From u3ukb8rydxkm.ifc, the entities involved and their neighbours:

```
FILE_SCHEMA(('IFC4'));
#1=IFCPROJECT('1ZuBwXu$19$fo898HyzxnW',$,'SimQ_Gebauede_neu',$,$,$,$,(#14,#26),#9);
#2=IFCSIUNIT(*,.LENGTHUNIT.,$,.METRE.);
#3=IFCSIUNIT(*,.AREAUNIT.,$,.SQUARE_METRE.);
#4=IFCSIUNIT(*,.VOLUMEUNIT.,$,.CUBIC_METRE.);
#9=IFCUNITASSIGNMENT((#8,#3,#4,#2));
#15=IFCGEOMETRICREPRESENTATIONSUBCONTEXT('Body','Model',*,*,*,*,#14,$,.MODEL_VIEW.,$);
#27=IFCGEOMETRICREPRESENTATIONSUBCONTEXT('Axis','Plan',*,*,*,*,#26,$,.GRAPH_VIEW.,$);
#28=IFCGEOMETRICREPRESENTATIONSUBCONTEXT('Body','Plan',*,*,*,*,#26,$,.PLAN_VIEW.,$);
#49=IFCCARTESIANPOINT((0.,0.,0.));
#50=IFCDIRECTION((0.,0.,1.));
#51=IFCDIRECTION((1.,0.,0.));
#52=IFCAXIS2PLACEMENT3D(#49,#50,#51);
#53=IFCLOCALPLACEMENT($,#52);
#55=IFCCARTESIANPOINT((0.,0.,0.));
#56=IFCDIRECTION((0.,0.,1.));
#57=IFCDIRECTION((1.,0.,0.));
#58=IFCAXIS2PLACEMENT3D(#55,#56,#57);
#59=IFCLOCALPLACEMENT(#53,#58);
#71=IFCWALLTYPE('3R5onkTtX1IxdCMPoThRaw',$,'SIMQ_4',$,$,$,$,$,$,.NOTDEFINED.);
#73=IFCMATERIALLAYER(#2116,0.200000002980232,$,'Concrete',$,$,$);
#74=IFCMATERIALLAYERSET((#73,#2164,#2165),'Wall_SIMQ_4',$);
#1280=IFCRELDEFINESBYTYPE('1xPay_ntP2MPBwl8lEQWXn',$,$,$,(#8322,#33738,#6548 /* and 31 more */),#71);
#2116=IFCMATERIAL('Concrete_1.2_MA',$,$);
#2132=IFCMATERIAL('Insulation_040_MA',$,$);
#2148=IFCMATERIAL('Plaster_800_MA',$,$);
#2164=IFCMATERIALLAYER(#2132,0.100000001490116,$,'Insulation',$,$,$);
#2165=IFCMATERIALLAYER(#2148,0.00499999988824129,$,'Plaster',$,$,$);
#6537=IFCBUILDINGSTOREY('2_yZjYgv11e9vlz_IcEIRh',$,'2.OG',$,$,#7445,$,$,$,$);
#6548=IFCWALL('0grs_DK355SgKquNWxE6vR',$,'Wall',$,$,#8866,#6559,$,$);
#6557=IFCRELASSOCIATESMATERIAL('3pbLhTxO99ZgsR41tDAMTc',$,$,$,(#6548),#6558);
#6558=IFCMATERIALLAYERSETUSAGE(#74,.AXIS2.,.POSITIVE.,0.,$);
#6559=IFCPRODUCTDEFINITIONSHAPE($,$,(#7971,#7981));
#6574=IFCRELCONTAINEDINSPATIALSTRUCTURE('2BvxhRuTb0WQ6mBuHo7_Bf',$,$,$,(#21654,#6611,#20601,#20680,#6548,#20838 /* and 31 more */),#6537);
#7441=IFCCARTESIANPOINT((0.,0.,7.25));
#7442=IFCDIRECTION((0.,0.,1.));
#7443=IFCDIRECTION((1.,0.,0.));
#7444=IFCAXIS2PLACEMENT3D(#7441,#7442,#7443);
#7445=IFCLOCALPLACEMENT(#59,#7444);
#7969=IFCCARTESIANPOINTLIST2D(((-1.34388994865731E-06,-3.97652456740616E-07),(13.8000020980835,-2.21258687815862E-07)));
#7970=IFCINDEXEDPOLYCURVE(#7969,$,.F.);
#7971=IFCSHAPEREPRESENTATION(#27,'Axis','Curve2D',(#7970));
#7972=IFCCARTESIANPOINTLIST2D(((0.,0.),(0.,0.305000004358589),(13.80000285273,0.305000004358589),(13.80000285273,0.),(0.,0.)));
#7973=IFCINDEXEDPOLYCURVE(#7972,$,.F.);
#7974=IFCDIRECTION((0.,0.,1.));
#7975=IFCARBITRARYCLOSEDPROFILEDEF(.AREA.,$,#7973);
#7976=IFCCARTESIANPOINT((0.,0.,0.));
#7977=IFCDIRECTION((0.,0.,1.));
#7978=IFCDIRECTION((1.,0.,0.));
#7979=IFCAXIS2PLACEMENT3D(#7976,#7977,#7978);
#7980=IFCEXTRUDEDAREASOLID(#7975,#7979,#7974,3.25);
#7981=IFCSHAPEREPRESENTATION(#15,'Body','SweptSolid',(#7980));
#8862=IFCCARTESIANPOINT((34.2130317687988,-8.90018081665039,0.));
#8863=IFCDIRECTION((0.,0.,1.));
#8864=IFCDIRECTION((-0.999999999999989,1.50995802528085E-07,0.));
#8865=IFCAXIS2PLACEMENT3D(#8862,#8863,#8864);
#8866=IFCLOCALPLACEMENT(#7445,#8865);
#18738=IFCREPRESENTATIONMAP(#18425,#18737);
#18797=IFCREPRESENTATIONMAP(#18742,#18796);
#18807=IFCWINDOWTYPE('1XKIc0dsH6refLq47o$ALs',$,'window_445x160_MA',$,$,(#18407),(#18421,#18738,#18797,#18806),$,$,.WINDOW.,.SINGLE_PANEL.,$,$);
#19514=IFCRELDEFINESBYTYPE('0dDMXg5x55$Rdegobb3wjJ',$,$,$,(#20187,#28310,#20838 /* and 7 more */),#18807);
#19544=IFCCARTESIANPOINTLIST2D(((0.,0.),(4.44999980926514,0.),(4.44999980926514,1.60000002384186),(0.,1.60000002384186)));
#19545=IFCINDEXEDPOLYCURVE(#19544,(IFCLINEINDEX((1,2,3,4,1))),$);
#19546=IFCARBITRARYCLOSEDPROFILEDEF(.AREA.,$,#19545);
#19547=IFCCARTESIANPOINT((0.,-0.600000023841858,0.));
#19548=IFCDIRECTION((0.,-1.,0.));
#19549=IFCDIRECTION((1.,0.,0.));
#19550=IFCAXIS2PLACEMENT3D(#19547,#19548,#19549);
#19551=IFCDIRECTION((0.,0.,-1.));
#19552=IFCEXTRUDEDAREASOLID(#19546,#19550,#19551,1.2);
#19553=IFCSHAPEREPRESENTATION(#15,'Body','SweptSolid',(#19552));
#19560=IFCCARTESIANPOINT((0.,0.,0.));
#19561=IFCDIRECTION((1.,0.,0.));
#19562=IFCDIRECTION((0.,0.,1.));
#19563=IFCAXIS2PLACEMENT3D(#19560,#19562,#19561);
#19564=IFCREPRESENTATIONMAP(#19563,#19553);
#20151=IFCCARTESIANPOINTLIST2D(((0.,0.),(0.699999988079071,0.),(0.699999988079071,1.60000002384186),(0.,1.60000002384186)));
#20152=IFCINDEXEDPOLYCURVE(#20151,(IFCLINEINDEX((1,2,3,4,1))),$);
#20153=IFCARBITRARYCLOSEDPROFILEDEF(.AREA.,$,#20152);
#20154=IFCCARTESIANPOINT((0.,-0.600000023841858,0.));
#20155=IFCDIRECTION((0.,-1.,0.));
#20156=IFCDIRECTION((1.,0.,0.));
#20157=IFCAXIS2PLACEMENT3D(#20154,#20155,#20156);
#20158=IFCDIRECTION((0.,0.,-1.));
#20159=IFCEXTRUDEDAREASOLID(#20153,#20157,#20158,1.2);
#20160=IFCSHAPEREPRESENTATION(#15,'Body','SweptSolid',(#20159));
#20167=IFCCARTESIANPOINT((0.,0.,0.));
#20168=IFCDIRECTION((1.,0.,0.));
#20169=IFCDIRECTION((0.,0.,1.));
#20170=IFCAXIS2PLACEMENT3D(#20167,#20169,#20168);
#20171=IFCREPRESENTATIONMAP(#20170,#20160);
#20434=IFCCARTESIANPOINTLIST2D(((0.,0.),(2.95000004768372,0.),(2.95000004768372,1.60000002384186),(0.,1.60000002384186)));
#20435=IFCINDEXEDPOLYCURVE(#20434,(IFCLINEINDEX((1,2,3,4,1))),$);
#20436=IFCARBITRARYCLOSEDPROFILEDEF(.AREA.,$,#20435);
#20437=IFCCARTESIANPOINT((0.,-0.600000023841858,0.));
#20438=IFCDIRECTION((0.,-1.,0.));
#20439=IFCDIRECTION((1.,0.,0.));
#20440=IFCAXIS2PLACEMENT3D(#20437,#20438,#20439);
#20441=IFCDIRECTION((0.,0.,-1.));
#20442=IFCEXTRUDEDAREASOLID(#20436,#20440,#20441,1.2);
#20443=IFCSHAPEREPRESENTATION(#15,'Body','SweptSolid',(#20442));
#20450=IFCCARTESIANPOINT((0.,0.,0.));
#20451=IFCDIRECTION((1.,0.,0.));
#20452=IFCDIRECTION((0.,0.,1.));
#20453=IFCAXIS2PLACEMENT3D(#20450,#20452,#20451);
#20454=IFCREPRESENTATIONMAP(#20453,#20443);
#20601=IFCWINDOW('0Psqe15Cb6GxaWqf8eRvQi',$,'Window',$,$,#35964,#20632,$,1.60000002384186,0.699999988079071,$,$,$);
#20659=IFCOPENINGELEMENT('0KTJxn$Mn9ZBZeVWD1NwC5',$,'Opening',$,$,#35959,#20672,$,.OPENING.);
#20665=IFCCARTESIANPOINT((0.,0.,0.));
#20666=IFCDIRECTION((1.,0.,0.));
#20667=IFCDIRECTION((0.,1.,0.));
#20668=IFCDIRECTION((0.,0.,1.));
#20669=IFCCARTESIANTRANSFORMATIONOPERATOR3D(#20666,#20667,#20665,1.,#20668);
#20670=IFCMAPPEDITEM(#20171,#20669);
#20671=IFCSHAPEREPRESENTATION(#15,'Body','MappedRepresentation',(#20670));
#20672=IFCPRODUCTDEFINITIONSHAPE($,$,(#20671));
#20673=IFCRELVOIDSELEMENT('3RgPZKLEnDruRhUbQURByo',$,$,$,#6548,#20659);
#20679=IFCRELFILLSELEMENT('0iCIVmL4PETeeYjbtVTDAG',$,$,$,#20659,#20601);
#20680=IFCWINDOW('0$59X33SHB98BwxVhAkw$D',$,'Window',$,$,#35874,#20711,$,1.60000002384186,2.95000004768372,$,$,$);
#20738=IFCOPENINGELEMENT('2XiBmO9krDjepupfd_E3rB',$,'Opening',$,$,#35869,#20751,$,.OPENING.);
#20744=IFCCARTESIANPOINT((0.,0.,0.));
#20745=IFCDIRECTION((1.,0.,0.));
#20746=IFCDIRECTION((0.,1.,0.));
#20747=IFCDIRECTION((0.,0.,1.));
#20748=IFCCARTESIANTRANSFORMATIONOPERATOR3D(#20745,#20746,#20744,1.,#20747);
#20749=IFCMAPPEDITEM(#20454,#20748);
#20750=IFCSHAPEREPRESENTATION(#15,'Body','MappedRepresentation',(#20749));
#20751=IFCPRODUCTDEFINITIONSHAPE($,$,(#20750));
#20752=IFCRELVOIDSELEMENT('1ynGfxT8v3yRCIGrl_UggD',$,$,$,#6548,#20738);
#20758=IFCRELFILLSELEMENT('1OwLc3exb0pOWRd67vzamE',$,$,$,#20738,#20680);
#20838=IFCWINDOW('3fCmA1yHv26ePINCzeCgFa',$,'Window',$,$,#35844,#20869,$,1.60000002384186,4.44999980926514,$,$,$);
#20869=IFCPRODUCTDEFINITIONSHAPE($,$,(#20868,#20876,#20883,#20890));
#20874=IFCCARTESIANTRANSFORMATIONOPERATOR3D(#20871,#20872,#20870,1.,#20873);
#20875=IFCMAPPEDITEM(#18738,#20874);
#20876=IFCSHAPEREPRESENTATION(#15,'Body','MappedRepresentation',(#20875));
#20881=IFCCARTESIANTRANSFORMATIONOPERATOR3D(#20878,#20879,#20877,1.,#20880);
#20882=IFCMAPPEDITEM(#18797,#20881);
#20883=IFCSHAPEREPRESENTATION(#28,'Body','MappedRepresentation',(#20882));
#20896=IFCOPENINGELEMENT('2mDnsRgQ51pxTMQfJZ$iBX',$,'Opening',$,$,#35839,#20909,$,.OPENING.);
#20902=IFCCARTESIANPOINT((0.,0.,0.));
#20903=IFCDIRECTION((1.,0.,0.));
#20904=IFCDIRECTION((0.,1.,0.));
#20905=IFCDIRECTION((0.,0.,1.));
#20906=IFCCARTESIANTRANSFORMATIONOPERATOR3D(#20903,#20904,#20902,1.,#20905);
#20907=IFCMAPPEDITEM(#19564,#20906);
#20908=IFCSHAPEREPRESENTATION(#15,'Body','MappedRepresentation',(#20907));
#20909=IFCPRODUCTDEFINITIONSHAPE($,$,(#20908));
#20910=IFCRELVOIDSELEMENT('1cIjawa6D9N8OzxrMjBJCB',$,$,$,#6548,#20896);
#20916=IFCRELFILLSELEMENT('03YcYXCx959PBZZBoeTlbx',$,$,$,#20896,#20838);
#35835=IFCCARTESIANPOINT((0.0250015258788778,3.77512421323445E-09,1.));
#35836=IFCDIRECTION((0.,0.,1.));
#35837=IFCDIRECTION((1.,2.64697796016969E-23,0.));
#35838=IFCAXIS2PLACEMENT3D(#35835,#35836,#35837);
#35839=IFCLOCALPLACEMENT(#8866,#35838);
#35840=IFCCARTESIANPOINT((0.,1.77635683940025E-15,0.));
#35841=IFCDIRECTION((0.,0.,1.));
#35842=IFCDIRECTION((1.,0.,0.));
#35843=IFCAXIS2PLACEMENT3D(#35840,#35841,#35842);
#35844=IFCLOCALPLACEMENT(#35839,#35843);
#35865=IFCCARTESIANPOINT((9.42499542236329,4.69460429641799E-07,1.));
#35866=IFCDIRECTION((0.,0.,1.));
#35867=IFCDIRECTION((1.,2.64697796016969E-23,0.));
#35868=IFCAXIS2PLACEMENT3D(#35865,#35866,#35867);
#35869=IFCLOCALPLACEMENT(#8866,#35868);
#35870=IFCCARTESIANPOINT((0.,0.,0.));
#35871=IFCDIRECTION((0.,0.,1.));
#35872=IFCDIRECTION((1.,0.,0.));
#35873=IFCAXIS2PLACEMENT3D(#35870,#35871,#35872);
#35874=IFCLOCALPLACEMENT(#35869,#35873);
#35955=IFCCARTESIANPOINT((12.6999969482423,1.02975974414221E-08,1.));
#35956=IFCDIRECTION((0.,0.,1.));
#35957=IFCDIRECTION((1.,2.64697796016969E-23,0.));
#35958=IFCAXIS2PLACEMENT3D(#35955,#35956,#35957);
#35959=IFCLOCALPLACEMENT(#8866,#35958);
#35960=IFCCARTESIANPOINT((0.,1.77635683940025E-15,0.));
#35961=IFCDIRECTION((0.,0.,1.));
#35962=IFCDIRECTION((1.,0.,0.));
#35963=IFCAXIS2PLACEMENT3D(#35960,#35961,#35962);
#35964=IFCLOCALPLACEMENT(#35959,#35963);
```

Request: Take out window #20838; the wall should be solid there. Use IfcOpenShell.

```python
import ifcopenshell
import ifcopenshell.api.feature
import ifcopenshell.api.root
import ifcopenshell.geom
import ifcopenshell.util.shape

model = ifcopenshell.open("u3ukb8rydxkm.ifc")
settings = ifcopenshell.geom.settings()


def volume(element):
    """Net volume in cubic metres, openings subtracted."""
    shape = ifcopenshell.geom.create_shape(settings, element)
    return ifcopenshell.util.shape.get_volume(shape.geometry)


window = model.by_id(20838)
opening = window.FillsVoids[0].RelatingOpeningElement
wall = opening.VoidsElements[0].RelatingBuildingElement
before = volume(wall)

ifcopenshell.api.root.remove_product(model, product=window)
ifcopenshell.api.feature.remove_feature(model, feature=opening)

after = volume(wall)

print(f"wall volume {before:.3f} -> {after:.3f} m3")

model.write("u3ukb8rydxkm_updated.ifc")
```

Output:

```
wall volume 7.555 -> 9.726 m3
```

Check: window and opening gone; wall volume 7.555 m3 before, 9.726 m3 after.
